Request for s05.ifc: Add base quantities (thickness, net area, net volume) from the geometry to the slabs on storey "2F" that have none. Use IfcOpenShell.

First a look at what the model holds.

```python
import ifcopenshell
import ifcopenshell.util.element
import ifcopenshell.util.unit

model = ifcopenshell.open("s05.ifc")
print(model.schema)
for unit_type in ("LENGTHUNIT", "AREAUNIT", "VOLUMEUNIT"):
    print(unit_type, ifcopenshell.util.unit.calculate_unit_scale(model, unit_type))
storey = next(s for s in model.by_type("IfcBuildingStorey") if s.Name == "2F")
slabs = [e for e in ifcopenshell.util.element.get_decomposition(storey) if e.is_a("IfcSlab")]
for e in sorted(slabs, key=lambda e: e.id()):
    print(e.id(), e.is_a(), e.Name, list(ifcopenshell.util.element.get_psets(e, qtos_only=True)), sep=" | ")
```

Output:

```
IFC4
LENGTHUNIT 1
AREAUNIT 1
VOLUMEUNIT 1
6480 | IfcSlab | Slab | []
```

```python
import ifcopenshell
import ifcopenshell.api.pset
import ifcopenshell.geom
import ifcopenshell.util.element
import ifcopenshell.util.shape
import ifcopenshell.util.unit

model = ifcopenshell.open("s05.ifc")
unit_scale = ifcopenshell.util.unit.calculate_unit_scale(model)
area_scale = ifcopenshell.util.unit.calculate_unit_scale(model, "AREAUNIT")
volume_scale = ifcopenshell.util.unit.calculate_unit_scale(model, "VOLUMEUNIT")
settings = ifcopenshell.geom.settings()

storey = next(s for s in model.by_type("IfcBuildingStorey") if s.Name == "2F")
slabs = [e for e in ifcopenshell.util.element.get_decomposition(storey) if e.is_a("IfcSlab")]

for e in sorted(slabs, key=lambda e: e.id()):
    if ifcopenshell.util.element.get_psets(e, qtos_only=True, should_inherit=False):
        continue
    # Geometry comes back in metres, in the element's own axes.
    shape = ifcopenshell.geom.create_shape(settings, e)
    values = {
        "Width": ifcopenshell.util.shape.get_z(shape.geometry) / unit_scale,
        "NetArea": ifcopenshell.util.shape.get_footprint_area(shape.geometry) / area_scale,
        "NetVolume": ifcopenshell.util.shape.get_volume(shape.geometry) / volume_scale,
    }
    qto = ifcopenshell.api.pset.add_qto(model, product=e, name="Qto_SlabBaseQuantities")
    ifcopenshell.api.pset.edit_qto(model, qto=qto, properties=values)
    print(e.id(), {k: round(v, 3) for k, v in values.items()})

model.write("s05_v2.ifc")
```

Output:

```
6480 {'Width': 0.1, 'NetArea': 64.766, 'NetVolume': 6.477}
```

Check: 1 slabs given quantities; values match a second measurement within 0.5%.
